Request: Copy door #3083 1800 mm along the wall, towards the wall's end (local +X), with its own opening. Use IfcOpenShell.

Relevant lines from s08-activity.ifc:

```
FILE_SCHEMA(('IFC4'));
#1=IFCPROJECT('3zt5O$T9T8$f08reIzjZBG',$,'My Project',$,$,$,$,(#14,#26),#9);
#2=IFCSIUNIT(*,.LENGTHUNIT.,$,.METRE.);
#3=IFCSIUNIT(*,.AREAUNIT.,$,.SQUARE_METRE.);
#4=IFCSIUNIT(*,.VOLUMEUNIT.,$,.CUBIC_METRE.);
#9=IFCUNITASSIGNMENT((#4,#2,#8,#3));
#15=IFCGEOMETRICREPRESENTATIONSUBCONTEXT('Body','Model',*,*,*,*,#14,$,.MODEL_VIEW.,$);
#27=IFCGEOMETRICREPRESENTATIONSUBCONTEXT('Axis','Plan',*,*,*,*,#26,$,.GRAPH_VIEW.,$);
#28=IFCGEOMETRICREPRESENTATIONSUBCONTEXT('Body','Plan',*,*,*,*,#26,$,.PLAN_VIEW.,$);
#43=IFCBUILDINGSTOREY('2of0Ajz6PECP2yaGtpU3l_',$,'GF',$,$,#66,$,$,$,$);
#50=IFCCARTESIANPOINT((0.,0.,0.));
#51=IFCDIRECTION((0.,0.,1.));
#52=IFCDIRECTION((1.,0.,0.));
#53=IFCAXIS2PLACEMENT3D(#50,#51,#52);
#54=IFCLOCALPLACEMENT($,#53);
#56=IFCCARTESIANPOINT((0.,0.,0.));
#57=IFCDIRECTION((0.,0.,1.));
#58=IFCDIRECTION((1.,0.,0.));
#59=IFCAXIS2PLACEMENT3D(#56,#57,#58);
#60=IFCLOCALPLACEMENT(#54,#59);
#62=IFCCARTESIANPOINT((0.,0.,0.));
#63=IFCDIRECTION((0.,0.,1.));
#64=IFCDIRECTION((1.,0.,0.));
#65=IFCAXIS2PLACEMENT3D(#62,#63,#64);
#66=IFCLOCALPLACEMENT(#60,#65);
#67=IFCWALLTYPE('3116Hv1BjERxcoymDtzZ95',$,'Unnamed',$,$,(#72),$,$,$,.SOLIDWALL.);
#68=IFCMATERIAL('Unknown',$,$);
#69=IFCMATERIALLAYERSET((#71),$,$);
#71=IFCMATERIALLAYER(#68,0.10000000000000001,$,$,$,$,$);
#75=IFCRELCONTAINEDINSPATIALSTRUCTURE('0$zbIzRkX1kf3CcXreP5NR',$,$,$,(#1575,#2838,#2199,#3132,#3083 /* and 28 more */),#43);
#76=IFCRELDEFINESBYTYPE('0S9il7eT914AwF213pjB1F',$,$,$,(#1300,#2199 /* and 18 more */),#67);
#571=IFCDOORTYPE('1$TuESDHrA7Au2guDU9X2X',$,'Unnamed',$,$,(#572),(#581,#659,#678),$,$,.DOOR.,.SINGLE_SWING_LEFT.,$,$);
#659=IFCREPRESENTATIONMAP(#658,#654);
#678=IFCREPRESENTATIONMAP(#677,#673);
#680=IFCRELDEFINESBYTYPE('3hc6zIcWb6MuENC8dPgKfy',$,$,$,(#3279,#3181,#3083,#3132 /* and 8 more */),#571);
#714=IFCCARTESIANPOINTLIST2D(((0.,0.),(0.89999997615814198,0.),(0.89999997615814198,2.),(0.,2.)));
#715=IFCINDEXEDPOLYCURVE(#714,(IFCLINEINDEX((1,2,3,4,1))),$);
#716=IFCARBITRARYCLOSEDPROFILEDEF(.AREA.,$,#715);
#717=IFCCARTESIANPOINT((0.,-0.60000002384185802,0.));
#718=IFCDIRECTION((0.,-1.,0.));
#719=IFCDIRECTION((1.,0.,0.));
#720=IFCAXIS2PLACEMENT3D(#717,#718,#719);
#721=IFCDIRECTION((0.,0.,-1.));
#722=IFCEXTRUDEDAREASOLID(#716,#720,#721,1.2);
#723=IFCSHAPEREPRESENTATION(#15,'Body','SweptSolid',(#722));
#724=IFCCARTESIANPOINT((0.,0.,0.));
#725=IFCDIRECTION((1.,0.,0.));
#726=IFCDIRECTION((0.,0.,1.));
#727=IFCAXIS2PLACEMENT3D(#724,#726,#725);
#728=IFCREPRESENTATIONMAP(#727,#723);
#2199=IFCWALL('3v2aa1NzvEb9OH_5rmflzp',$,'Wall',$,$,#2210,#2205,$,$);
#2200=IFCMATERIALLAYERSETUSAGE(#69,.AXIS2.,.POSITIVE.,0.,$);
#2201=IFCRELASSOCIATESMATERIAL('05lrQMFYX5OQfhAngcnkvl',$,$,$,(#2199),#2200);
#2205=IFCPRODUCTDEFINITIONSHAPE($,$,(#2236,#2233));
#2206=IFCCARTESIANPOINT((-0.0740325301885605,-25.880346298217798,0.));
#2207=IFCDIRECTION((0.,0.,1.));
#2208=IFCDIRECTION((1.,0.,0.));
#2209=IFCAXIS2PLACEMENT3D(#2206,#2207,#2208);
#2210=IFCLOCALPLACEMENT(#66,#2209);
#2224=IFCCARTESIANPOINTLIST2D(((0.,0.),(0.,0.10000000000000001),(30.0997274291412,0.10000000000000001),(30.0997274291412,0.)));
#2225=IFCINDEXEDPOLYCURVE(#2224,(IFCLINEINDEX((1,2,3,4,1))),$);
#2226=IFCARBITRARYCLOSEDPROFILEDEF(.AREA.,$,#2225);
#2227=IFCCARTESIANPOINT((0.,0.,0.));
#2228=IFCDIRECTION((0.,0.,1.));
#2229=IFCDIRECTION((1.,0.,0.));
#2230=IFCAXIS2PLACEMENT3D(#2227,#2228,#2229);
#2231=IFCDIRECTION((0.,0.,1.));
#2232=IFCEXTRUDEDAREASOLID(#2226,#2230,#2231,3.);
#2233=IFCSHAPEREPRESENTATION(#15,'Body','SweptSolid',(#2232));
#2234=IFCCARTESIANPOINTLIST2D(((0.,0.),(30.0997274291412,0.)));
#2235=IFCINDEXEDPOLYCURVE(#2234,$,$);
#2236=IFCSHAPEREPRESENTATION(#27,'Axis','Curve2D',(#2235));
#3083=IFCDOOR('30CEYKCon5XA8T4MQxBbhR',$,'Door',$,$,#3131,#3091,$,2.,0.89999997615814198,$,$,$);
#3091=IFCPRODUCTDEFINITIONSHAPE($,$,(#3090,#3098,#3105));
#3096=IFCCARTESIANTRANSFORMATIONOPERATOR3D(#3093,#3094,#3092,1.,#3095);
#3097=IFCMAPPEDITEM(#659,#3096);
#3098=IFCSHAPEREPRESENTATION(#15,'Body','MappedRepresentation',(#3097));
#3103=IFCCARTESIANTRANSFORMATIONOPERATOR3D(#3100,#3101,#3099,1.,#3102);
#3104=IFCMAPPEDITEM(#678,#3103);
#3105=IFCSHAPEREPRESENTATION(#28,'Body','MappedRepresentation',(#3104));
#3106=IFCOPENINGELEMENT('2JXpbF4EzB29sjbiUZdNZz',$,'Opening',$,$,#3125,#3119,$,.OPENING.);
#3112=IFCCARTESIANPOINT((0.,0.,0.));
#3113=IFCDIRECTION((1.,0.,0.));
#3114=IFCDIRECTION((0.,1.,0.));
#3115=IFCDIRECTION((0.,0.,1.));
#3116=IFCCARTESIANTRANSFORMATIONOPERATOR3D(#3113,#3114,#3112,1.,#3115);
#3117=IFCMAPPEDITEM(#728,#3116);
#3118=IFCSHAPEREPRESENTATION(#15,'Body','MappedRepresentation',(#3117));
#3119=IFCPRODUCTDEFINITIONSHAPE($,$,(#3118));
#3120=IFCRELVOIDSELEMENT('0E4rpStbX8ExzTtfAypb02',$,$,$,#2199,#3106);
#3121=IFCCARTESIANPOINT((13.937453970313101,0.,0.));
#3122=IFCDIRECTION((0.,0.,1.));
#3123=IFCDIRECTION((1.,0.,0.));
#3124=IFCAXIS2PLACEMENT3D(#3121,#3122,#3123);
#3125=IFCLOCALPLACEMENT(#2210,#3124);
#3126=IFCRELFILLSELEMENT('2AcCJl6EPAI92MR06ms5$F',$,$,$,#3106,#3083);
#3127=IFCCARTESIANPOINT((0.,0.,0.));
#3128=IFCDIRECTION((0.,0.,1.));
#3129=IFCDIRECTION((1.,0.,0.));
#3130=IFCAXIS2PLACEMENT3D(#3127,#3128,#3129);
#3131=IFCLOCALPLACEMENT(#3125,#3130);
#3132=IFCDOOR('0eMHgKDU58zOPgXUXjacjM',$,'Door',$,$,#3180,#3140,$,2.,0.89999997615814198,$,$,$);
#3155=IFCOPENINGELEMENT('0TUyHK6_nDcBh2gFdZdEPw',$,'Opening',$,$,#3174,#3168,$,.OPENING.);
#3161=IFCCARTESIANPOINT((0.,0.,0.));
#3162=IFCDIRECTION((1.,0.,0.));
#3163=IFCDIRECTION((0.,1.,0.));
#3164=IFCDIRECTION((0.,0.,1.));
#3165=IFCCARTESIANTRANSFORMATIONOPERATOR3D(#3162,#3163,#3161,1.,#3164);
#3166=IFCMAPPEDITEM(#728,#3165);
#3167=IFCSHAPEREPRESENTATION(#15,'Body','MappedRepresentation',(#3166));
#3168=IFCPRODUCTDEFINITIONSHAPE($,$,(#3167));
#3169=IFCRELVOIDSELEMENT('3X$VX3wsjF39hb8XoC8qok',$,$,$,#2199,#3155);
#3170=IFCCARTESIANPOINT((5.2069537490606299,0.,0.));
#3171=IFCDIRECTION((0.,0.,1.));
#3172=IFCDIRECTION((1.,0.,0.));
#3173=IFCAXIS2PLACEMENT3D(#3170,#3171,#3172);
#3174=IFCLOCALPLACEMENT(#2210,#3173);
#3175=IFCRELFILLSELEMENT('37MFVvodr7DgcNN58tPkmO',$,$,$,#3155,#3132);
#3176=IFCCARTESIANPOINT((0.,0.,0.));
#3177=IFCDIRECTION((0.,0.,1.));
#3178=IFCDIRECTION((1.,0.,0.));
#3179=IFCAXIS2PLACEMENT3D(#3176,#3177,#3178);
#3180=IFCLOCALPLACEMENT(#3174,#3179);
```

```python
import ifcopenshell
import ifcopenshell.api.feature
import ifcopenshell.api.geometry
import ifcopenshell.api.root
import ifcopenshell.geom
import ifcopenshell.util.element
import ifcopenshell.util.placement
import ifcopenshell.util.shape
import ifcopenshell.util.unit

model = ifcopenshell.open("s08-activity.ifc")
unit_scale = ifcopenshell.util.unit.calculate_unit_scale(model)
settings = ifcopenshell.geom.settings()


def volume(element):
    """Net volume in cubic metres, openings subtracted."""
    shape = ifcopenshell.geom.create_shape(settings, element)
    return ifcopenshell.util.shape.get_volume(shape.geometry)


door = model.by_guid("30CEYKCon5XA8T4MQxBbhR")
opening = door.FillsVoids[0].RelatingOpeningElement
wall = opening.VoidsElements[0].RelatingBuildingElement
before = volume(wall)
shift = ifcopenshell.util.placement.get_local_placement(wall.ObjectPlacement)[:3, 0] * 1.8 / unit_scale

# copy_class copies the void relationship, type, container and properties, but no geometry.
new_opening = ifcopenshell.api.root.copy_class(model, product=opening)
new_opening.Representation = ifcopenshell.util.element.copy_deep(
    model, opening.Representation, exclude=["IfcGeometricRepresentationContext", "IfcRepresentationMap"]
)
new_door = ifcopenshell.api.root.copy_class(model, product=door)
new_door.Representation = ifcopenshell.util.element.copy_deep(
    model, door.Representation, exclude=["IfcGeometricRepresentationContext", "IfcRepresentationMap"]
)
ifcopenshell.api.feature.add_filling(model, opening=new_opening, element=new_door)

for old, new in ((opening, new_opening), (door, new_door)):
    matrix = ifcopenshell.util.placement.get_local_placement(old.ObjectPlacement)
    matrix[:3, 3] += shift
    ifcopenshell.api.geometry.edit_object_placement(model, product=new, matrix=matrix, is_si=False)

after = volume(wall)

print(f"wall volume {before:.3f} -> {after:.3f} m3")

model.write("s08-activity_rev.ifc")
```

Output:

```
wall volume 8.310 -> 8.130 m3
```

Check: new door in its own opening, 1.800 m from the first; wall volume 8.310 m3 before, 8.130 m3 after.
